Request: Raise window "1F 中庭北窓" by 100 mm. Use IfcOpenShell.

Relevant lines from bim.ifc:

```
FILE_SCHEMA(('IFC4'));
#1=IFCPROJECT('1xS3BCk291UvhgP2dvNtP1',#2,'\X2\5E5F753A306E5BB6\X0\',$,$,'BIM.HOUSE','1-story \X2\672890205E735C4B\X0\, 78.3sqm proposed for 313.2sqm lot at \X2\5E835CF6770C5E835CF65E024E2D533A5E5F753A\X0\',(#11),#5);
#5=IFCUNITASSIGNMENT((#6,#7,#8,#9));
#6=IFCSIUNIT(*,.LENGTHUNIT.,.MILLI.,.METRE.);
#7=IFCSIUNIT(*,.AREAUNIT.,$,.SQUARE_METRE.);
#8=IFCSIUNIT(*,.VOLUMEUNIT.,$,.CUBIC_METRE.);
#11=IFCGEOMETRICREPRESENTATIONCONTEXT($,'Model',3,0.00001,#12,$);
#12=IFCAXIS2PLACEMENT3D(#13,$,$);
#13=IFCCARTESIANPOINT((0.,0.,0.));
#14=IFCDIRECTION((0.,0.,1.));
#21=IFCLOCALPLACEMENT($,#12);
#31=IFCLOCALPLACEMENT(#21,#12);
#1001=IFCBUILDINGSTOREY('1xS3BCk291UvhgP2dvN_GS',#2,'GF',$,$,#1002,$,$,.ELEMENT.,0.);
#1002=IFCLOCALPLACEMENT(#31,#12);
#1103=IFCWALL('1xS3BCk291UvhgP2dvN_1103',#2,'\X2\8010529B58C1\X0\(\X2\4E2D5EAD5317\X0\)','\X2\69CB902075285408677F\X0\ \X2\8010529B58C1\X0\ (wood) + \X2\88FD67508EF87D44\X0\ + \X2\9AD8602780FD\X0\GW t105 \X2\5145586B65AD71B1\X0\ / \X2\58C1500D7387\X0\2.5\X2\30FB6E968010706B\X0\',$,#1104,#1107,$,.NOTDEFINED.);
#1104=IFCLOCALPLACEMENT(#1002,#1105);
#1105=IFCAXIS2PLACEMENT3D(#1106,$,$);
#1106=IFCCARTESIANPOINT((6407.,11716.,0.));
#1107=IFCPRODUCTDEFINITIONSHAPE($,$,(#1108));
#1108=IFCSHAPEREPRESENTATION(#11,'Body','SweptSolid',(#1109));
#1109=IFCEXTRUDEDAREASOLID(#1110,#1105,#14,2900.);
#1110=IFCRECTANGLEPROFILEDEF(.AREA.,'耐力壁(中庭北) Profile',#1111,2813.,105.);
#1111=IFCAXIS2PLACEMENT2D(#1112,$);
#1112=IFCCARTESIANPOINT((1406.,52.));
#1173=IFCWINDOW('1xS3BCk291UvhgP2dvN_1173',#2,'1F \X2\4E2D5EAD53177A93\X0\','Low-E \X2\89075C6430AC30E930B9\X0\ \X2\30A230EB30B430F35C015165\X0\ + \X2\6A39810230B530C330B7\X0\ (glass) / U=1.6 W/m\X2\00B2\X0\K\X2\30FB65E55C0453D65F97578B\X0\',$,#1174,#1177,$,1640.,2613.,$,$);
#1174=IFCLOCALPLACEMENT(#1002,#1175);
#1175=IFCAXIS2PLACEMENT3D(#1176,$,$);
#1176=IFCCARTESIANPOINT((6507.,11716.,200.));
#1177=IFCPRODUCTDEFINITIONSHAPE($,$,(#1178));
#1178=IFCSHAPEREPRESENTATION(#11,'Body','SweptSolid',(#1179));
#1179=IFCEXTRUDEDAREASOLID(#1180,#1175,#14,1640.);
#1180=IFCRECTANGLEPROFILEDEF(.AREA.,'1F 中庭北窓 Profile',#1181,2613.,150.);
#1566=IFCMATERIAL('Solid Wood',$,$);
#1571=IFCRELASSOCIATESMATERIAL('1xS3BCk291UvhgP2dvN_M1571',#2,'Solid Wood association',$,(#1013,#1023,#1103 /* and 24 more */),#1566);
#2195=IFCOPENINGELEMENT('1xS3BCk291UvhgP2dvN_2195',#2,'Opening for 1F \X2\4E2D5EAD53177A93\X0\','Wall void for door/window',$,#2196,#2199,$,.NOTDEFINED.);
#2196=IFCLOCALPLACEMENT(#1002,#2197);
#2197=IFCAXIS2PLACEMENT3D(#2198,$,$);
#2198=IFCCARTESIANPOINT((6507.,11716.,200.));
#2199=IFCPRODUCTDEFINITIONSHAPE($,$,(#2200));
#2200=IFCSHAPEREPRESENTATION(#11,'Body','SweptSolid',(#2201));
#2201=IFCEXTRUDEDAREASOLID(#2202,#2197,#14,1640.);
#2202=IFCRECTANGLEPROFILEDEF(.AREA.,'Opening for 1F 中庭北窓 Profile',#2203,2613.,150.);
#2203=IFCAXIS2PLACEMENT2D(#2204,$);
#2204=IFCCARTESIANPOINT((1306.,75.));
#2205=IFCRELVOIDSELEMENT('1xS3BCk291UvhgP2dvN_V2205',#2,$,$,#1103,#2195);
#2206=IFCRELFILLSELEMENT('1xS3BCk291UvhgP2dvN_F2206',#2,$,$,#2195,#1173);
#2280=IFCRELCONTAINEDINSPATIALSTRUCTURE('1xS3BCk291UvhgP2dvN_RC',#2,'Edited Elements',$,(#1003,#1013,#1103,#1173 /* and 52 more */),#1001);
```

```python
import numpy as np
import ifcopenshell
import ifcopenshell.api.geometry
import ifcopenshell.util.placement
import ifcopenshell.util.unit

model = ifcopenshell.open("bim.ifc")
unit_scale = ifcopenshell.util.unit.calculate_unit_scale(model)

window = model.by_id(1173)
opening = window.FillsVoids[0].RelatingOpeningElement
dz = 0.1 / unit_scale

shift = np.array([0.0, 0.0, dz])
# The window is not placed relative to its opening, so move both.
for product in (opening, window):
    matrix = ifcopenshell.util.placement.get_local_placement(product.ObjectPlacement)
    matrix[:3, 3] += shift
    ifcopenshell.api.geometry.edit_object_placement(model, product=product, matrix=matrix, is_si=False)

print(f"moved by {dz * unit_scale:+.3f} m")

model.write("bim_updated.ifc")
```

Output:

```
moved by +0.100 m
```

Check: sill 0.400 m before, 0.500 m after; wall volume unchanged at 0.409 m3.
